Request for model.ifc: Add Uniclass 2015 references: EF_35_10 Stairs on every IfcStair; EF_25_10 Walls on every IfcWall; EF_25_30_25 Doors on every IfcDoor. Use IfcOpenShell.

First a look at what the model holds.

```python
import ifcopenshell

model = ifcopenshell.open("model.ifc")
print(model.schema)
print("classifications:", [c.Name for c in model.by_type("IfcClassification")])
for ifc_class in ("IfcDoor", "IfcRoof", "IfcStair", "IfcWall", "IfcWindow"):
    print(ifc_class, len(model.by_type(ifc_class)))
```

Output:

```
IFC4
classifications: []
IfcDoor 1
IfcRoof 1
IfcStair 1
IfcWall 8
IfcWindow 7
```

```python
import ifcopenshell
import ifcopenshell.api.classification

model = ifcopenshell.open("model.ifc")

system = ifcopenshell.api.classification.add_classification(model, classification="Uniclass 2015")

codes = {
    "IfcStair": ("EF_35_10", "Stairs"),
    "IfcWall": ("EF_25_10", "Walls"),
    "IfcDoor": ("EF_25_30_25", "Doors"),
}
for ifc_class, (code, name) in codes.items():
    products = model.by_type(ifc_class)
    ifcopenshell.api.classification.add_reference(
        model, products=products, classification=system, identification=code, name=name
    )
    print(code, len(products))

model.write("model-out.ifc")
```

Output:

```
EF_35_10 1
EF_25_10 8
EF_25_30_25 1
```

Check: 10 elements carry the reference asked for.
